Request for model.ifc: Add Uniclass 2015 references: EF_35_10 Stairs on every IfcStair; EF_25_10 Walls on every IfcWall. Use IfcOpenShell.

First a look at what the model holds.

```python
import ifcopenshell

model = ifcopenshell.open("model.ifc")
print(model.schema)
print("classifications:", [c.Name for c in model.by_type("IfcClassification")])
for ifc_class in ("IfcDoor", "IfcRoof", "IfcStair", "IfcWall", "IfcWindow"):
    print(ifc_class, len(model.by_type(ifc_class)))
```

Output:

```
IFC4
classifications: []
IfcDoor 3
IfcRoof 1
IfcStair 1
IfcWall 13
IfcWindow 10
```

```python
import ifcopenshell
import ifcopenshell.api.classification

model = ifcopenshell.open("model.ifc")

system = ifcopenshell.api.classification.add_classification(model, classification="Uniclass 2015")

codes = {
    "IfcStair": ("EF_35_10", "Stairs"),
    "IfcWall": ("EF_25_10", "Walls"),
}
for ifc_class, (code, name) in codes.items():
    products = model.by_type(ifc_class)
    ifcopenshell.api.classification.add_reference(
        model, products=products, classification=system, identification=code, name=name
    )
    print(code, len(products))

model.write("model_edited.ifc")
```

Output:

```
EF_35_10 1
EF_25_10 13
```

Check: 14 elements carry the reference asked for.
